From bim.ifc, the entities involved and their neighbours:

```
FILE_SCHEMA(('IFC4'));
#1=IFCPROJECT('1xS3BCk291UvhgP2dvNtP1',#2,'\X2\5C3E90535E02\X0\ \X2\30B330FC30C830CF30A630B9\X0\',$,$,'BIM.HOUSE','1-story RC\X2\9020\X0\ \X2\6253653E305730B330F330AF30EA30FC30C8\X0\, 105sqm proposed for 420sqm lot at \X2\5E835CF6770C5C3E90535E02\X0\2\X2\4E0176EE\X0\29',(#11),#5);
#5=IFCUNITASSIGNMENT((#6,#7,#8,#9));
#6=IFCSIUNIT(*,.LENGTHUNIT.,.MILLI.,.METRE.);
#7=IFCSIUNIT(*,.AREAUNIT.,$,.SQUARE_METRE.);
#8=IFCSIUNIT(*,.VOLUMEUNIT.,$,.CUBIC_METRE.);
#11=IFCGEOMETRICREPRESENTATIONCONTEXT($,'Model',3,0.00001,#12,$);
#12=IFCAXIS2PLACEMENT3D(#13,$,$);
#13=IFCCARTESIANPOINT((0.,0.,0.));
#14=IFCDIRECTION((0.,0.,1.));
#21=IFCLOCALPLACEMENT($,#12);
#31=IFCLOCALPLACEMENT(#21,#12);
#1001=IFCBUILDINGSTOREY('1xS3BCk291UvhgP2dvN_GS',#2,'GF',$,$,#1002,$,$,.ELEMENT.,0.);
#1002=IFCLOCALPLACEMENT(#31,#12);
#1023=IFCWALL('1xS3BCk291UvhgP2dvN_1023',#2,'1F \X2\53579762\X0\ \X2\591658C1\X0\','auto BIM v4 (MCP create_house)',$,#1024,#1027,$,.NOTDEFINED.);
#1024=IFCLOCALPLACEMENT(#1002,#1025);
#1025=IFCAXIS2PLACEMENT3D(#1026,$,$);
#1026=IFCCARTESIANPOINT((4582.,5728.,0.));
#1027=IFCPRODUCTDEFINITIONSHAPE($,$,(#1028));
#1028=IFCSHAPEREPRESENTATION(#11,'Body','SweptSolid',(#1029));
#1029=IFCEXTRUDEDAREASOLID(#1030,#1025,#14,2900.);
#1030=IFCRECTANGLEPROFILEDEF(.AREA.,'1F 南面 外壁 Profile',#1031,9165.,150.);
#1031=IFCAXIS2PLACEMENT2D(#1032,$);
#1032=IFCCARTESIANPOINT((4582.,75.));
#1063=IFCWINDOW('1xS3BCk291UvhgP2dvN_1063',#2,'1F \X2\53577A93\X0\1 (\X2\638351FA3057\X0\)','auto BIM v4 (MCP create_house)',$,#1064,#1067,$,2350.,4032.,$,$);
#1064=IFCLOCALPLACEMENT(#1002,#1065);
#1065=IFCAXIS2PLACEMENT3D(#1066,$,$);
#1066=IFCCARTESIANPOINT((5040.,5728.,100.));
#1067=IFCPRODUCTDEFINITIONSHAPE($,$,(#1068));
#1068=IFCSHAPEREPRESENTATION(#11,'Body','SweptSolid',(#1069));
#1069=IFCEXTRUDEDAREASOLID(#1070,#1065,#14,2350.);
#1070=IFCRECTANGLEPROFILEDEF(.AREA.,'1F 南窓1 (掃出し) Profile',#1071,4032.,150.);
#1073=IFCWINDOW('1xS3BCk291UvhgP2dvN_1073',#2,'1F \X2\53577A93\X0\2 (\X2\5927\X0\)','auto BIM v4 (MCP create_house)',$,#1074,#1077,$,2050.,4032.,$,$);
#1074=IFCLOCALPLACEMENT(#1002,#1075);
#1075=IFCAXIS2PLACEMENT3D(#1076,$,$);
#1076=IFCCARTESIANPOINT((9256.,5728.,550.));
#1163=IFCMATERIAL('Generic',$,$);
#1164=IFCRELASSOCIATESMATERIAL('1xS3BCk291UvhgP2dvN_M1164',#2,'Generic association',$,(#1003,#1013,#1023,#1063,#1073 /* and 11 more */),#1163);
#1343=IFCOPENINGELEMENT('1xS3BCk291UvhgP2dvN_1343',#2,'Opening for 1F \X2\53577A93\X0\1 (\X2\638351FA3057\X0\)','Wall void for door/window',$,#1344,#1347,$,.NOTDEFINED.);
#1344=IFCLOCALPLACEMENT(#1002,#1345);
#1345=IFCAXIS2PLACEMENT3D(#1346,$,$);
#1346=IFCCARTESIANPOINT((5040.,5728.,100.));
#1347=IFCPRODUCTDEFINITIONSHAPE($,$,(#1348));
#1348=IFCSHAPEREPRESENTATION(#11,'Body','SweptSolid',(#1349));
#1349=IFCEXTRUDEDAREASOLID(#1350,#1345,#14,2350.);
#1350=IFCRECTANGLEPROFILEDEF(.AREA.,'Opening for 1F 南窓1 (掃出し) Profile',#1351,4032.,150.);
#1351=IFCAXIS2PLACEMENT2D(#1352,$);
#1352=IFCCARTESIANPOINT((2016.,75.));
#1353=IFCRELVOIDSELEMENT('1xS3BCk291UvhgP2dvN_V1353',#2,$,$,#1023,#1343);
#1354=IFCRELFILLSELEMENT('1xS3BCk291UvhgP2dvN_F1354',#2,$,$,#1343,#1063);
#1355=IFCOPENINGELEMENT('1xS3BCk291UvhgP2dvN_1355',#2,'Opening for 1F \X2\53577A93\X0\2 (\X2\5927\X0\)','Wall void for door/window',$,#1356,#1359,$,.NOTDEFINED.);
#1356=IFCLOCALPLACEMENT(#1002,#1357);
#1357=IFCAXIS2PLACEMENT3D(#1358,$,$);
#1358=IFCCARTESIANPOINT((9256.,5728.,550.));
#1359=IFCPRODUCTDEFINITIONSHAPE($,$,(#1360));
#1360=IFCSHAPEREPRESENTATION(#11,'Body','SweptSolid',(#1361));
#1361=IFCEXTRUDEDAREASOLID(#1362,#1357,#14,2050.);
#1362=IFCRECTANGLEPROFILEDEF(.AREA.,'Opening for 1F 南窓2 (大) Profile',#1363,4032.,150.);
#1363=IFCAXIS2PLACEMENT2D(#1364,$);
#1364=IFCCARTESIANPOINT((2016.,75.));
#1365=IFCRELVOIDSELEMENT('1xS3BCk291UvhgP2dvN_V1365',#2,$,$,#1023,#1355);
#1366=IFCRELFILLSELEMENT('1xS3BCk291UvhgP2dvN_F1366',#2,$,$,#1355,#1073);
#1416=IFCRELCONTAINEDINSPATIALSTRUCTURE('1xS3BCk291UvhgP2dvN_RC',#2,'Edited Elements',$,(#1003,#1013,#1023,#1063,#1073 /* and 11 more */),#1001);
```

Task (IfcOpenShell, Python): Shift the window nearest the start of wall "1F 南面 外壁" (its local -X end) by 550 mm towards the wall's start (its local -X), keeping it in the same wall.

```python
import ifcopenshell
import ifcopenshell.api.geometry
import ifcopenshell.util.placement

model = ifcopenshell.open("bim.ifc")

window = model.by_id(1063)
opening = window.FillsVoids[0].RelatingOpeningElement
wall = opening.VoidsElements[0].RelatingBuildingElement

wall_matrix = ifcopenshell.util.placement.get_local_placement(wall.ObjectPlacement)
shift = wall_matrix[:3, 0] * -550.0
before = ifcopenshell.util.placement.get_local_placement(window.ObjectPlacement)[:3, 3].copy()

# The window is not placed relative to its opening, so move both.
for product in (opening, window):
    matrix = ifcopenshell.util.placement.get_local_placement(product.ObjectPlacement)
    matrix[:3, 3] += shift
    ifcopenshell.api.geometry.edit_object_placement(model, product=product, matrix=matrix, is_si=False)

after = ifcopenshell.util.placement.get_local_placement(window.ObjectPlacement)[:3, 3]
print("window moved by", (after - before).round(3) + 0.0)

model.write("bim_updated.ifc")
```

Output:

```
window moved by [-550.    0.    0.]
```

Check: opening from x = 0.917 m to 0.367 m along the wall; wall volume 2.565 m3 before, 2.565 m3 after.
